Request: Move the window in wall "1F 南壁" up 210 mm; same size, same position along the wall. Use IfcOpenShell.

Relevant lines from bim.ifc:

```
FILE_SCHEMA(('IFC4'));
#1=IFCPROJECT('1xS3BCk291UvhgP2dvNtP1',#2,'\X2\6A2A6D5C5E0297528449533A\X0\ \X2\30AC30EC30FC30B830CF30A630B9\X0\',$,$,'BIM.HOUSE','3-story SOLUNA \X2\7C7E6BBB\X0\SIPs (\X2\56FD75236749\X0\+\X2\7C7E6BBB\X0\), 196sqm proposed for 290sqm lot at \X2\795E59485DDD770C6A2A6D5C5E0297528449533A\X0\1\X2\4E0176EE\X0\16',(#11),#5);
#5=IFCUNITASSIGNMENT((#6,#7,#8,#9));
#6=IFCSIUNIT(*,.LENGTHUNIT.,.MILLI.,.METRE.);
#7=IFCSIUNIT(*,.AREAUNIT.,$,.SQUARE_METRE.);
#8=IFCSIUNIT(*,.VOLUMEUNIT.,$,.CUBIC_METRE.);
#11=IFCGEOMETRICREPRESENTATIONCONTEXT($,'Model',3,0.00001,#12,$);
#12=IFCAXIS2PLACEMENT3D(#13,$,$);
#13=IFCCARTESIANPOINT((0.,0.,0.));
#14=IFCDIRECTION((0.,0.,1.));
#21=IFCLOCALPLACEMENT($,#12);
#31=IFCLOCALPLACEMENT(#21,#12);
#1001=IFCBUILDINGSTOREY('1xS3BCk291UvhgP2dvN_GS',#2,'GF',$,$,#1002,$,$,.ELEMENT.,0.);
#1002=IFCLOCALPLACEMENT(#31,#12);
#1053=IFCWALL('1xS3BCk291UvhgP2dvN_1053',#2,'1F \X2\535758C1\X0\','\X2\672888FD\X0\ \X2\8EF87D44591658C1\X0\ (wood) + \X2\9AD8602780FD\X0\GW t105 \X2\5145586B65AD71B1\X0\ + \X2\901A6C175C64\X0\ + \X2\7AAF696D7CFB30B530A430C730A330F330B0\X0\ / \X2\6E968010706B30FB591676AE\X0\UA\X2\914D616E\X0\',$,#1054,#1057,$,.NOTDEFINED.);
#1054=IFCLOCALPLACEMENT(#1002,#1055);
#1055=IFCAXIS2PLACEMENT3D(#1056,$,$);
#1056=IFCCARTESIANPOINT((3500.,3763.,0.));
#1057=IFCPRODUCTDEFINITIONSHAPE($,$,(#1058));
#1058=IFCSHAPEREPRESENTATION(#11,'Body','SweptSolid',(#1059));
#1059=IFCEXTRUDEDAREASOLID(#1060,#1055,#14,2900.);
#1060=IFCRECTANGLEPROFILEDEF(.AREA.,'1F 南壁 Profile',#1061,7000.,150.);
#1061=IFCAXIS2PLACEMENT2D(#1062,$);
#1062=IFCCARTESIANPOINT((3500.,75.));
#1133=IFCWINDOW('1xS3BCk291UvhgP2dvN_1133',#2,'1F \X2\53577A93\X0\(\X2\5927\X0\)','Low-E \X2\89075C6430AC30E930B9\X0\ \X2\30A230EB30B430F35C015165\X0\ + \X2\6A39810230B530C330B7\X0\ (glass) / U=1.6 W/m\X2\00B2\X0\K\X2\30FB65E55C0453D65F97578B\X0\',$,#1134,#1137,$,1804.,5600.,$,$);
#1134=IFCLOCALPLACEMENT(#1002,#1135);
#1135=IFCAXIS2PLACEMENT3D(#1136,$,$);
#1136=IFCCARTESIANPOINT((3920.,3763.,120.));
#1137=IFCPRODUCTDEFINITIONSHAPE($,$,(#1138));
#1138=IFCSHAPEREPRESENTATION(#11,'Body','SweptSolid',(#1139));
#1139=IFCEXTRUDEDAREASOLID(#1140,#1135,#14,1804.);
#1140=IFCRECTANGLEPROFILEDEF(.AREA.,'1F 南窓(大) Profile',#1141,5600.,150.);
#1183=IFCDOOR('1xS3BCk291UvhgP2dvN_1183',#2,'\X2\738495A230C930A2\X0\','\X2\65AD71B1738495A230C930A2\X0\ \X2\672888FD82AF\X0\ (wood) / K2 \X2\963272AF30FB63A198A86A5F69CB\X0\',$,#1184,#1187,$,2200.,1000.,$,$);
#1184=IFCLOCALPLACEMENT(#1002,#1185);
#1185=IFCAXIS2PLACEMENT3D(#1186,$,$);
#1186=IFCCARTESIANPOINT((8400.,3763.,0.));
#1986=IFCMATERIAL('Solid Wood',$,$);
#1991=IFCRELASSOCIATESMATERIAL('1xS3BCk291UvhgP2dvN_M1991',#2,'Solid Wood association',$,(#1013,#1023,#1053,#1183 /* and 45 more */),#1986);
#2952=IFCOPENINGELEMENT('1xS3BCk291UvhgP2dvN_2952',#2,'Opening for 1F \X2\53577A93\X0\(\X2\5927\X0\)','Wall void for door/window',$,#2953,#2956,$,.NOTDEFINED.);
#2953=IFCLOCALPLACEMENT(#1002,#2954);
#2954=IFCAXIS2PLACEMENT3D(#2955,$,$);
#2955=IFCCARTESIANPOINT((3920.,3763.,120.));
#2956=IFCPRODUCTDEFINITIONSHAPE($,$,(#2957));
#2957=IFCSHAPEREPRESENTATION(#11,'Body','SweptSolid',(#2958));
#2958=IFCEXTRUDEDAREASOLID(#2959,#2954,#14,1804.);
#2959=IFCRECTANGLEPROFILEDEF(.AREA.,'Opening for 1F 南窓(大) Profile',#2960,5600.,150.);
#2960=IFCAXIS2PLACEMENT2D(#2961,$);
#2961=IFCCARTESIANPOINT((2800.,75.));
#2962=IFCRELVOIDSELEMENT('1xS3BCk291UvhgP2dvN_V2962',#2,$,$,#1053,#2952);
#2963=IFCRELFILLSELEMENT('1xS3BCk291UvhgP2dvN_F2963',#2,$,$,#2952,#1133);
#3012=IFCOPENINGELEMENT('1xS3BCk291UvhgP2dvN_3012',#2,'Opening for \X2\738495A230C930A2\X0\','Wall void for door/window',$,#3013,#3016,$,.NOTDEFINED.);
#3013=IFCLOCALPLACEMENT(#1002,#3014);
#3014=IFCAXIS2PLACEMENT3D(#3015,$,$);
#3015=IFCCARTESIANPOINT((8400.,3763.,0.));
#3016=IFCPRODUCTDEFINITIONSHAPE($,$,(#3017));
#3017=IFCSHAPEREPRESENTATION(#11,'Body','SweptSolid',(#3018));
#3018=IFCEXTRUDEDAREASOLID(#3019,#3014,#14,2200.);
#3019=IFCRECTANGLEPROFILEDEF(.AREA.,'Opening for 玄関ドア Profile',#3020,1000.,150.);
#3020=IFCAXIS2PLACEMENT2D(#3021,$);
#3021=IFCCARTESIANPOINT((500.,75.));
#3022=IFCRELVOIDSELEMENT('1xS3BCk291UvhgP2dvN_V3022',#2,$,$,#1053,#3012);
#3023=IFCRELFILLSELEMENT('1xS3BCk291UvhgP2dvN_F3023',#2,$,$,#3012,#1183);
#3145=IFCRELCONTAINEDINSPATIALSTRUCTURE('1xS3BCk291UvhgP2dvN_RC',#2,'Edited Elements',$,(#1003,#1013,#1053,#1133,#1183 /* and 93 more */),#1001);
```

```python
import numpy as np
import ifcopenshell
import ifcopenshell.api.geometry
import ifcopenshell.util.placement
import ifcopenshell.util.unit

model = ifcopenshell.open("bim.ifc")
unit_scale = ifcopenshell.util.unit.calculate_unit_scale(model)

window = model.by_guid("1xS3BCk291UvhgP2dvN_1133")
opening = window.FillsVoids[0].RelatingOpeningElement
dz = 0.21 / unit_scale

shift = np.array([0.0, 0.0, dz])
# The window is not placed relative to its opening, so move both.
for product in (opening, window):
    matrix = ifcopenshell.util.placement.get_local_placement(product.ObjectPlacement)
    matrix[:3, 3] += shift
    ifcopenshell.api.geometry.edit_object_placement(model, product=product, matrix=matrix, is_si=False)

print(f"moved by {dz * unit_scale:+.3f} m")

model.write("bim_v2.ifc")
```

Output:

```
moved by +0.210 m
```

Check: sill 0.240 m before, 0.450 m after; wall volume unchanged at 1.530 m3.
